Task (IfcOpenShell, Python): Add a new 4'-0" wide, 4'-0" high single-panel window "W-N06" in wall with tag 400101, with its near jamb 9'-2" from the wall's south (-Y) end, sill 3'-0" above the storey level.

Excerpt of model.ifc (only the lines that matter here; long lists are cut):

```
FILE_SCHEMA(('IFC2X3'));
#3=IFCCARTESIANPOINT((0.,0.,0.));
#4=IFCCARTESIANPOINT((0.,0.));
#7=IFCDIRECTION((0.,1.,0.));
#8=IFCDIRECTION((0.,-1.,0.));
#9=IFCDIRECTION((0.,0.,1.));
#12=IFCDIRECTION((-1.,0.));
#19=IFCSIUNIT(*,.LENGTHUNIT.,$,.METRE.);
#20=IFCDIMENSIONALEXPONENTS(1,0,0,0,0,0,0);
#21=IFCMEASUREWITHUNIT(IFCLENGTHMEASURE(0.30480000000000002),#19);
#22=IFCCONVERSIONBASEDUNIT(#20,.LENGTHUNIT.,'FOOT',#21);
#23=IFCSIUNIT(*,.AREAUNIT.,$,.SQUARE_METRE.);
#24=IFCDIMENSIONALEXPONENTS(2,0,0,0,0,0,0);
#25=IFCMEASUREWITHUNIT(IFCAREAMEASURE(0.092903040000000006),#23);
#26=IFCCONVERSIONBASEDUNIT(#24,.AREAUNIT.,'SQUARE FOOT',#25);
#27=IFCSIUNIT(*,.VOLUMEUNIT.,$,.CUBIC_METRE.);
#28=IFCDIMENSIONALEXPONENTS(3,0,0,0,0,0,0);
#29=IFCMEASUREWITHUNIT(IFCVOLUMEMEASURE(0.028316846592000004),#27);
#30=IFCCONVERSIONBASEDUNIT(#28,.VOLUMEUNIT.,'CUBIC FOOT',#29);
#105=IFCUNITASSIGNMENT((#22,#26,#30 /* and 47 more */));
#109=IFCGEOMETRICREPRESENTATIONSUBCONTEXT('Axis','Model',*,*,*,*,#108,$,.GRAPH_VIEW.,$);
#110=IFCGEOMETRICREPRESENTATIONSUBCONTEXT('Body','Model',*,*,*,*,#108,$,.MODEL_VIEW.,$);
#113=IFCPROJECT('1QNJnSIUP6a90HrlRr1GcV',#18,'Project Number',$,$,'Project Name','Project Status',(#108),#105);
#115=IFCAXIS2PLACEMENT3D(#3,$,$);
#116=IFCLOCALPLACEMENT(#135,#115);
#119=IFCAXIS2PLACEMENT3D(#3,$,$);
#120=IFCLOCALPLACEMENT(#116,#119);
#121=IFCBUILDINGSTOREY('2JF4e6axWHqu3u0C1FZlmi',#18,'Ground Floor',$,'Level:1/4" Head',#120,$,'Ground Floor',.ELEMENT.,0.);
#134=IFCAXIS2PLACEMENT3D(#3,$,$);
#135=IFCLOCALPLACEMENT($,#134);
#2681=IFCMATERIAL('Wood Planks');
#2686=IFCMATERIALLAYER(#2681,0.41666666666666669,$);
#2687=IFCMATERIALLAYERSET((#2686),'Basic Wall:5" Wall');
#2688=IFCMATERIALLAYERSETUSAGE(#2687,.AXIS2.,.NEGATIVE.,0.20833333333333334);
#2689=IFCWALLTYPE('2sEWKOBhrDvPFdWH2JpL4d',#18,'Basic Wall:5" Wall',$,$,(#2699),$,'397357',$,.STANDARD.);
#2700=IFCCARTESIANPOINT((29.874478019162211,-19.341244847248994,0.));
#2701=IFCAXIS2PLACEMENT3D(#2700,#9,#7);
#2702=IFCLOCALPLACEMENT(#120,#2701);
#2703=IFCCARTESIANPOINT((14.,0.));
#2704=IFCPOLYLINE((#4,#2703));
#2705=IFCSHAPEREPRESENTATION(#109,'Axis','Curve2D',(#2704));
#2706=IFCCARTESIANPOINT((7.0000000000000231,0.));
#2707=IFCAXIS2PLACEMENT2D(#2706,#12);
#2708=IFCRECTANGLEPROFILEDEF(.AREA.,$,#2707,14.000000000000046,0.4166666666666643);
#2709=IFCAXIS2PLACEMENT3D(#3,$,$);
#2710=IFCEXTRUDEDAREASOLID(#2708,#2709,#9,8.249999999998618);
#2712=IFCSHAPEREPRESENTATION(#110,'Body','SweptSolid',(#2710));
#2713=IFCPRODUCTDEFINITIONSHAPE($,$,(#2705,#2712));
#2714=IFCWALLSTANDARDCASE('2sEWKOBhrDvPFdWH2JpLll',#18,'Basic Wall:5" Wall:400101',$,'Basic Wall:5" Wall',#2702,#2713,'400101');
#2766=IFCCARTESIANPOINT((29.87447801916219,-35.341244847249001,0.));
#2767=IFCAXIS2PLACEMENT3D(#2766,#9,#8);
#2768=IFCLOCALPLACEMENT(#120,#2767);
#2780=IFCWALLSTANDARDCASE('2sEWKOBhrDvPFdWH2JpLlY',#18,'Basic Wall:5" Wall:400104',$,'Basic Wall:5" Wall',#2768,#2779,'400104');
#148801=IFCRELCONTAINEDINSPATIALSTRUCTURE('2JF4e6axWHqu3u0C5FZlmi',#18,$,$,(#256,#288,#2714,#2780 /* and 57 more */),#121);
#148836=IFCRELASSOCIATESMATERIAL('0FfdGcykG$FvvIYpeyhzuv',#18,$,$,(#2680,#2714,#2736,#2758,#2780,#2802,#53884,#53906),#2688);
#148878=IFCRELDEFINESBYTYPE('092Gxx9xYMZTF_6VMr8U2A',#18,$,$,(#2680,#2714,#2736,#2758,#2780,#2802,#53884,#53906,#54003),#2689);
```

```python
import numpy as np
import ifcopenshell
import ifcopenshell.api.feature
import ifcopenshell.api.geometry
import ifcopenshell.api.root
import ifcopenshell.api.spatial
import ifcopenshell.api.type
import ifcopenshell.geom
import ifcopenshell.util.element
import ifcopenshell.util.placement
import ifcopenshell.util.representation
import ifcopenshell.util.shape
import ifcopenshell.util.unit

model = ifcopenshell.open("model.ifc")
unit_scale = ifcopenshell.util.unit.calculate_unit_scale(model)
settings = ifcopenshell.geom.settings()


def volume(element):
    """Net volume in cubic metres, openings subtracted."""
    shape = ifcopenshell.geom.create_shape(settings, element)
    return ifcopenshell.util.shape.get_volume(shape.geometry)


wall = model.by_guid("2sEWKOBhrDvPFdWH2JpLll")
storey = ifcopenshell.util.element.get_container(wall, ifc_class="IfcBuildingStorey")
context = ifcopenshell.util.representation.get_context(model, "Model", "Body", "MODEL_VIEW")
before = volume(wall)

width, height, from_end, sill = 1.2192, 1.2192, 2.794, 0.9144  # metres

# The wall runs along its own X axis, and the end named is its -X end.
wall_shape = ifcopenshell.geom.create_shape(settings, wall)
x, y, z = ifcopenshell.util.shape.get_vertices(wall_shape.geometry).T
start = x.min() + from_end
face, thickness = float(y.min()), float(y.max() - y.min())
wall_matrix = ifcopenshell.util.placement.get_local_placement(wall.ObjectPlacement)
level = ifcopenshell.util.placement.get_local_placement(storey.ObjectPlacement)[2, 3]


def in_wall(x, y):
    """Placement at x, y metres in the wall's axes, at sill height."""
    matrix = wall_matrix.copy()
    matrix[:, 3] = wall_matrix @ np.array([x / unit_scale, y / unit_scale, 0.0, 1.0])
    matrix[2, 3] = level + sill / unit_scale
    return matrix


# Opening: a box that overshoots both wall faces by 50 mm.
opening = ifcopenshell.api.root.create_entity(model, ifc_class="IfcOpeningElement")
box = ifcopenshell.api.geometry.add_wall_representation(
    model, context=context, length=width, height=height, thickness=thickness + 0.1
)
ifcopenshell.api.geometry.assign_representation(model, product=opening, representation=box)
ifcopenshell.api.geometry.edit_object_placement(model, product=opening, matrix=in_wall(start, face - 0.05), is_si=False)
ifcopenshell.api.feature.add_feature(model, feature=opening, element=wall)

window = ifcopenshell.api.root.create_entity(model, ifc_class="IfcWindow", name="W-N06")
window.OverallWidth, window.OverallHeight = width / unit_scale, height / unit_scale
body = ifcopenshell.api.geometry.add_window_representation(
    model,
    context=context,
    overall_width=window.OverallWidth,
    overall_height=window.OverallHeight,
    partition_type="SINGLE_PANEL",
)
ifcopenshell.api.geometry.assign_representation(model, product=window, representation=body)
ifcopenshell.api.spatial.assign_container(model, products=[window], relating_structure=storey)
fills = ifcopenshell.api.feature.add_filling(model, opening=opening, element=window)
fills.OwnerHistory = window.OwnerHistory  # required in IFC2X3

# IFC2X3 keeps the operation on the window style.
style = ifcopenshell.api.root.create_entity(model, ifc_class="IfcWindowStyle", name="W-N06")
style.OperationType, style.ConstructionType = "SINGLE_PANEL", "NOTDEFINED"
style.ParameterTakesPrecedence = style.Sizeable = False
ifcopenshell.api.type.assign_type(model, related_objects=[window], relating_type=style)

# Centre the window in the wall's thickness.
ifcopenshell.api.geometry.edit_object_placement(model, product=window, matrix=in_wall(start, face), is_si=False)
window_shape = ifcopenshell.geom.create_shape(settings, window)
depth = ifcopenshell.util.shape.get_vertices(window_shape.geometry)[:, 1]
offset = face + thickness / 2 - (depth.min() + depth.max()) / 2
ifcopenshell.api.geometry.edit_object_placement(model, product=window, matrix=in_wall(start, offset), is_si=False)

after = volume(wall)

print(f"wall volume {before:.3f} -> {after:.3f} m3")

model.write("model_edited.ifc")
```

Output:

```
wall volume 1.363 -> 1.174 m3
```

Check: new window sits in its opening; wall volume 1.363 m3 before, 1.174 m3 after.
